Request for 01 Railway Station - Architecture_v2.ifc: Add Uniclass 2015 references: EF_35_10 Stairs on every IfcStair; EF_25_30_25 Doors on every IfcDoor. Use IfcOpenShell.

First a look at what the model holds.

```python
import ifcopenshell

model = ifcopenshell.open("01 Railway Station - Architecture_v2.ifc")
print(model.schema)
print("classifications:", [c.Name for c in model.by_type("IfcClassification")])
for ifc_class in ("IfcDoor", "IfcRoof", "IfcStair", "IfcWall", "IfcWindow"):
    print(ifc_class, len(model.by_type(ifc_class)))
```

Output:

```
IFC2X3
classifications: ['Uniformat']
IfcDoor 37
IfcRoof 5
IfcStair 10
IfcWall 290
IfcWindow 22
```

```python
import ifcopenshell
import ifcopenshell.api.classification

model = ifcopenshell.open("01 Railway Station - Architecture_v2.ifc")

# IFC2X3 requires Source and Edition and has no link from the project to the system.
system = model.create_entity("IfcClassification", Source="NBS", Edition="2015", Name="Uniclass 2015")

codes = {
    "IfcStair": ("EF_35_10", "Stairs"),
    "IfcDoor": ("EF_25_30_25", "Doors"),
}
for ifc_class, (code, name) in codes.items():
    products = model.by_type(ifc_class)
    ifcopenshell.api.classification.add_reference(
        model, products=products, classification=system, identification=code, name=name
    )
    print(code, len(products))

model.write("01 Railway Station - Architecture_v2_rev.ifc")
```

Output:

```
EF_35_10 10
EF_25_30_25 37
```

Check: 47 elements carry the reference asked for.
